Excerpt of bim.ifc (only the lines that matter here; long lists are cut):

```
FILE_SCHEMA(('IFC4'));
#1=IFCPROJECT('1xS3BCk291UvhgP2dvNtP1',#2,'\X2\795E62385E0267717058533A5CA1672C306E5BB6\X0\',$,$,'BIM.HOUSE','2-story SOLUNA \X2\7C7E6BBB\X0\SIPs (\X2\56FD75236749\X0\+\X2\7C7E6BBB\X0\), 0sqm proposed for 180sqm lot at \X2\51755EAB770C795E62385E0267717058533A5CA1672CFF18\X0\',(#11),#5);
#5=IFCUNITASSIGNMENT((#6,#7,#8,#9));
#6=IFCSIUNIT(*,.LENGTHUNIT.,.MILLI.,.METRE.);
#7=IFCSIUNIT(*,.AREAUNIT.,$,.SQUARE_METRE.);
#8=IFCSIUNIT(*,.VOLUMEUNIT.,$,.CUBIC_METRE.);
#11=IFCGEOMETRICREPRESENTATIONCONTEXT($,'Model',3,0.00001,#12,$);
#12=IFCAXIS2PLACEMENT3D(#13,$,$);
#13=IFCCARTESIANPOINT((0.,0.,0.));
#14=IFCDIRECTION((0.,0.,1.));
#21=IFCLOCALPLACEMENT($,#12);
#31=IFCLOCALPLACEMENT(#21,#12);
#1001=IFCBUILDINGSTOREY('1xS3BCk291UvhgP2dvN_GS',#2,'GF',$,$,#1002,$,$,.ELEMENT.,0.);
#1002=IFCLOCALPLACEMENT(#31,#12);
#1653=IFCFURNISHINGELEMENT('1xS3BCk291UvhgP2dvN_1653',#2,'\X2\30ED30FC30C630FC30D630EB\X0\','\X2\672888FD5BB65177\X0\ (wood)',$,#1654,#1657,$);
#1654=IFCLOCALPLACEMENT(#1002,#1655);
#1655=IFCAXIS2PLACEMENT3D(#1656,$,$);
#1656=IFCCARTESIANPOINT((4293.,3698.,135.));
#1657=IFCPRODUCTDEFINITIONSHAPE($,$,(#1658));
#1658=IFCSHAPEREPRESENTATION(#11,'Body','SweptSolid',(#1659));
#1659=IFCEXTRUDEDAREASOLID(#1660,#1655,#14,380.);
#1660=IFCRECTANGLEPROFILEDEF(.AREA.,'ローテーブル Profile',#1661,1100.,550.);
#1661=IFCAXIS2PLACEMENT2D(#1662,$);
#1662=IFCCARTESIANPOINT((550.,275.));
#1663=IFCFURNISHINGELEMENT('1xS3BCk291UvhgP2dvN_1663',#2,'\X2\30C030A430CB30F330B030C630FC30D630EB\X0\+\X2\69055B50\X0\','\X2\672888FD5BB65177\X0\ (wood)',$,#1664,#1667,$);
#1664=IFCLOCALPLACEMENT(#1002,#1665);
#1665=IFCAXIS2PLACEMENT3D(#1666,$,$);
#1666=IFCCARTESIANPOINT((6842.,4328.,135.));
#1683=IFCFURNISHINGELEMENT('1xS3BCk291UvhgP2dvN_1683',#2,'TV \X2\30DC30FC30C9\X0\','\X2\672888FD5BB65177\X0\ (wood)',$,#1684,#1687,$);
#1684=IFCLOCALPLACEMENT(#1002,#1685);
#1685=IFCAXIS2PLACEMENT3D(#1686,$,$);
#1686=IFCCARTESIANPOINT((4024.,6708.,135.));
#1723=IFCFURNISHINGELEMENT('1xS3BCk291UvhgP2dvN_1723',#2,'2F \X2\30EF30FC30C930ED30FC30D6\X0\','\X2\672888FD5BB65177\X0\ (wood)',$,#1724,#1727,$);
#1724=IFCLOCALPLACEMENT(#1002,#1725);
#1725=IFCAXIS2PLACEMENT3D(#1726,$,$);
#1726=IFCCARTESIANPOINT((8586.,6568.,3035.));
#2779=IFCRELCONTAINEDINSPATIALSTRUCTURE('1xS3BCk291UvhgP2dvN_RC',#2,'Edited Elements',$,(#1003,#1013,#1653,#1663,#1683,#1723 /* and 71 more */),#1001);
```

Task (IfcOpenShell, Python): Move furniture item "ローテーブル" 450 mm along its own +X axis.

```python
import ifcopenshell
import ifcopenshell.api.geometry
import ifcopenshell.util.placement
import ifcopenshell.util.unit

model = ifcopenshell.open("bim.ifc")
unit_scale = ifcopenshell.util.unit.calculate_unit_scale(model)

item = model.by_guid("1xS3BCk291UvhgP2dvN_1653")
matrix = ifcopenshell.util.placement.get_local_placement(item.ObjectPlacement)
matrix[:3, 3] += matrix[:3, 0] * 0.45 / unit_scale
ifcopenshell.api.geometry.edit_object_placement(model, product=item, matrix=matrix, is_si=False)

print(ifcopenshell.util.placement.get_local_placement(item.ObjectPlacement).round(3) + 0.0)

model.write("bim_updated.ifc")
```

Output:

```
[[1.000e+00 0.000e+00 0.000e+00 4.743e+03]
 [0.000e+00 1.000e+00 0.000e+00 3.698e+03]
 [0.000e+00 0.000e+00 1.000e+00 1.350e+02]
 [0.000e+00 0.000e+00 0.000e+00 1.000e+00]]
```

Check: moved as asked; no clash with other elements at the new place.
